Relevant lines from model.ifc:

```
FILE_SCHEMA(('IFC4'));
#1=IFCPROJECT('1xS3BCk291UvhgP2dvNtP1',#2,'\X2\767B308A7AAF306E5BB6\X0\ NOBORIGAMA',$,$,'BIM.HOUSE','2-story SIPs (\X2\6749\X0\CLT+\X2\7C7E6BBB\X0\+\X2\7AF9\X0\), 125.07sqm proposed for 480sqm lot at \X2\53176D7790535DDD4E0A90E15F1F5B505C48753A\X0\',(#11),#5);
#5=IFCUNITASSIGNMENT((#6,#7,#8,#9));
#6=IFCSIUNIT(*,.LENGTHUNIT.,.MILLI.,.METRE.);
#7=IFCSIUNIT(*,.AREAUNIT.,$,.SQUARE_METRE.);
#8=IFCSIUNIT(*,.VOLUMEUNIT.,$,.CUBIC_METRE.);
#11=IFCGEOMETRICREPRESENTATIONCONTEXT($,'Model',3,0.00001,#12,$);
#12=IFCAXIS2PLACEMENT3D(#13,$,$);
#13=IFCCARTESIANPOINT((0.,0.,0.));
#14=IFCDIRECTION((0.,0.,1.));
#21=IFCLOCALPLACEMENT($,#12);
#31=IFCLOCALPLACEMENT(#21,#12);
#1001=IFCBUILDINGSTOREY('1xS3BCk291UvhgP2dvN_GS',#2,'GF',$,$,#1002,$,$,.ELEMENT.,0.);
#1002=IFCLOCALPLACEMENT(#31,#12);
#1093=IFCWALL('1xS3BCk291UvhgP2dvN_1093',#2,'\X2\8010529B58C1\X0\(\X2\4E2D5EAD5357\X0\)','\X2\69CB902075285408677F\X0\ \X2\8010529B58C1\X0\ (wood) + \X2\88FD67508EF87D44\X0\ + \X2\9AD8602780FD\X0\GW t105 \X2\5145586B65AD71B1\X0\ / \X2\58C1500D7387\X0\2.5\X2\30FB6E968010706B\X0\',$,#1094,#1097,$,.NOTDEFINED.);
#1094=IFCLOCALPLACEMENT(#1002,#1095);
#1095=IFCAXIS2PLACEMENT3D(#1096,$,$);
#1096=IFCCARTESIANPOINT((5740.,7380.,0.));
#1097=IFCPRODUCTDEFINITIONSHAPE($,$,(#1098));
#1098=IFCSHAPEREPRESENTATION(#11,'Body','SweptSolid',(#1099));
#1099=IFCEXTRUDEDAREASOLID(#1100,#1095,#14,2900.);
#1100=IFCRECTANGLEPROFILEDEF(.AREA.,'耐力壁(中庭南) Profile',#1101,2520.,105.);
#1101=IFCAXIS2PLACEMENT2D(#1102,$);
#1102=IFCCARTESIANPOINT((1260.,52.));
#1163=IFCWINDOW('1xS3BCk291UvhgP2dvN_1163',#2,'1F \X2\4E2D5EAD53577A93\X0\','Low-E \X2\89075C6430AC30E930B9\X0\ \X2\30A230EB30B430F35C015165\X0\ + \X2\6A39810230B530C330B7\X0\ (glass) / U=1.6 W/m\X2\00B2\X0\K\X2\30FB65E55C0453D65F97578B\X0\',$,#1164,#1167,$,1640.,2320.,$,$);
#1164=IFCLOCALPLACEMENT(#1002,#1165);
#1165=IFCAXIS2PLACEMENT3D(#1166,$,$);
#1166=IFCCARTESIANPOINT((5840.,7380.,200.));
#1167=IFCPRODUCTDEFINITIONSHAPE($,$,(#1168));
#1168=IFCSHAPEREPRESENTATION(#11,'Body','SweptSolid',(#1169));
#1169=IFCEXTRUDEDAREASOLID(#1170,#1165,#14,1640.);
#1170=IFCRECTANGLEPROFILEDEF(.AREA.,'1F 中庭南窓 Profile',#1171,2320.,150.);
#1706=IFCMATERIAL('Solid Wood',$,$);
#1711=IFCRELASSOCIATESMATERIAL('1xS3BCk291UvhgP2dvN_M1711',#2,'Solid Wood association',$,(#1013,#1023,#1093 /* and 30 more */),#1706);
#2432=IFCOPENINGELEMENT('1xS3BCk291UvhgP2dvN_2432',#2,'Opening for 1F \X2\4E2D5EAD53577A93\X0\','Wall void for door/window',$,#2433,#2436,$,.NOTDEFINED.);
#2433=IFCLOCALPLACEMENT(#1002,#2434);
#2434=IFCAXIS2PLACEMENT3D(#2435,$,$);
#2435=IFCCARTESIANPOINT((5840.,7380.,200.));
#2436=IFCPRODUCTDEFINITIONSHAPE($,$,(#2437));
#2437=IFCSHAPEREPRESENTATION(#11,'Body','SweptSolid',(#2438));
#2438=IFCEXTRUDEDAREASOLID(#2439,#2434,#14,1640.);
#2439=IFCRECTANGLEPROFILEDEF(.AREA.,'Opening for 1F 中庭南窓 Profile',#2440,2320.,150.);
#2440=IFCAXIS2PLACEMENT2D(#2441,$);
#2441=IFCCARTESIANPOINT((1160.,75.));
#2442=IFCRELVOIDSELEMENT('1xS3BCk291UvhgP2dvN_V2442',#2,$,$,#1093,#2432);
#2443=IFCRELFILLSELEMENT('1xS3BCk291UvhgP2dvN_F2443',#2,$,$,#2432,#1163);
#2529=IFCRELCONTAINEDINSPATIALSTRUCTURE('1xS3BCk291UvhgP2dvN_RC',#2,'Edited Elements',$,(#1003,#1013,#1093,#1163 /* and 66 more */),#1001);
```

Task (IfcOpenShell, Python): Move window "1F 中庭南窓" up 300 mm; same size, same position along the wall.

```python
import numpy as np
import ifcopenshell
import ifcopenshell.api.geometry
import ifcopenshell.util.placement
import ifcopenshell.util.unit

model = ifcopenshell.open("model.ifc")
unit_scale = ifcopenshell.util.unit.calculate_unit_scale(model)

window = model.by_guid("1xS3BCk291UvhgP2dvN_1163")
opening = window.FillsVoids[0].RelatingOpeningElement
dz = 300.0

shift = np.array([0.0, 0.0, dz])
# The window is not placed relative to its opening, so move both.
for product in (opening, window):
    matrix = ifcopenshell.util.placement.get_local_placement(product.ObjectPlacement)
    matrix[:3, 3] += shift
    ifcopenshell.api.geometry.edit_object_placement(model, product=product, matrix=matrix, is_si=False)

print(f"moved by {dz * unit_scale:+.3f} m")

model.write("model-out.ifc")
```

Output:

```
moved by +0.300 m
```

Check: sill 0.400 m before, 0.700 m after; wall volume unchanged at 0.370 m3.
